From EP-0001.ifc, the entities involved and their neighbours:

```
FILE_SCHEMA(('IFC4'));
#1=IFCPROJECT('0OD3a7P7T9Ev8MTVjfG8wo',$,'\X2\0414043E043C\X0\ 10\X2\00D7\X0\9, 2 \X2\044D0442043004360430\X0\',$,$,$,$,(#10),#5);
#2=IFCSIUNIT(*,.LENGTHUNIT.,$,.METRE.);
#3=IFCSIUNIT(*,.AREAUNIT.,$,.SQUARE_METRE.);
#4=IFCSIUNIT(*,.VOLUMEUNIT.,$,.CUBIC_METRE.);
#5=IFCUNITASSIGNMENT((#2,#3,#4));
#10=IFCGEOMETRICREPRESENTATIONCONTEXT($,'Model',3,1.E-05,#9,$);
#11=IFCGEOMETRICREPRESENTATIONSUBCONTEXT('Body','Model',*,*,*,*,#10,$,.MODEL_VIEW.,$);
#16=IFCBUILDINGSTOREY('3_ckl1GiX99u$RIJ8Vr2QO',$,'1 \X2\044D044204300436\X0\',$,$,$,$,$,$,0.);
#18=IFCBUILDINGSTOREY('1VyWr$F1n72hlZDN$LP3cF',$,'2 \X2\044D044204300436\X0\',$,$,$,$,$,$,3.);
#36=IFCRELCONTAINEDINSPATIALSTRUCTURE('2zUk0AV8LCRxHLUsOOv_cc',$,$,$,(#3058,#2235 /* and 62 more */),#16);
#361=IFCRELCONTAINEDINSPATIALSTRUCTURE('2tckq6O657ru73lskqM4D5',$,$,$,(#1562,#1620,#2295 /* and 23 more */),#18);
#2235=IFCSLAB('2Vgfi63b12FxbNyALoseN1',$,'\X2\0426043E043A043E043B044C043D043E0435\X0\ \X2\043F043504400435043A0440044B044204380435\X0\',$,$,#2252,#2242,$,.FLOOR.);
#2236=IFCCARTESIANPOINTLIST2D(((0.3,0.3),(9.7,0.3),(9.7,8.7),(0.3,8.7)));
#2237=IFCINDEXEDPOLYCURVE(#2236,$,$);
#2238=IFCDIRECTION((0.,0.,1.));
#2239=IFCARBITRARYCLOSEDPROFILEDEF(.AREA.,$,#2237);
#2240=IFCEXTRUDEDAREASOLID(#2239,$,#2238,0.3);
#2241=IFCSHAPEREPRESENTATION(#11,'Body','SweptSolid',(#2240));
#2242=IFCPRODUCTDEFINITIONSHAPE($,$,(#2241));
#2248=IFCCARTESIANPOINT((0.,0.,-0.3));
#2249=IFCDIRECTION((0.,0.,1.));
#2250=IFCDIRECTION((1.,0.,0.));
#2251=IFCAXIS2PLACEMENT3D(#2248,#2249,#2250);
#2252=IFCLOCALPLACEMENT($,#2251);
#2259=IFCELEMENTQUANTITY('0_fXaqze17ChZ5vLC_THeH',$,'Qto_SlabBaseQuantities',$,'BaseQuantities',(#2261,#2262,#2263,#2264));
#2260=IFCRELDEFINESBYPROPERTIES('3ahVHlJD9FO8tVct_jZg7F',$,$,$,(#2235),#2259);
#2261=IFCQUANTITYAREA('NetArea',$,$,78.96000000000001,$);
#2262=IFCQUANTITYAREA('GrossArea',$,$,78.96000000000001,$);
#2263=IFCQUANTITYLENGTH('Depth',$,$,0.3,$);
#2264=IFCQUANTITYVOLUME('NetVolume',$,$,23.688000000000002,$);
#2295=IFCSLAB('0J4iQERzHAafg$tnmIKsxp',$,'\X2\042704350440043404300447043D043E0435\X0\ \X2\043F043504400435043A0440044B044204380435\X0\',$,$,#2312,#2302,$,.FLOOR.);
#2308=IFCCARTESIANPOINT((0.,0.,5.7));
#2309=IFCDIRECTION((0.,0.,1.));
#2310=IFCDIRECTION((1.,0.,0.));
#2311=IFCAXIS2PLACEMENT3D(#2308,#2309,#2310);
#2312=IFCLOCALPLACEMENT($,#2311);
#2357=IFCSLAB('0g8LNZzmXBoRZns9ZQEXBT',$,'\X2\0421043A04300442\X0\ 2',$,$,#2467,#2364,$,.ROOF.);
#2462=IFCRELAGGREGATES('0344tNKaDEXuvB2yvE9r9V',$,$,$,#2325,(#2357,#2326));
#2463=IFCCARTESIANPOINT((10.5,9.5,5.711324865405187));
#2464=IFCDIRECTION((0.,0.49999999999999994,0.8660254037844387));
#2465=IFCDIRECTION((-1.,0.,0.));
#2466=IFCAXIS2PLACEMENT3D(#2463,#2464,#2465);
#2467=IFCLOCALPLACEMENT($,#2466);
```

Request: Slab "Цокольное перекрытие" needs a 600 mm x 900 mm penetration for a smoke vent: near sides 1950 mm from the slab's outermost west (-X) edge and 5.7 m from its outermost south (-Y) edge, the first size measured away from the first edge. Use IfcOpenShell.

```python
import numpy as np
import ifcopenshell
import ifcopenshell.api.feature
import ifcopenshell.api.geometry
import ifcopenshell.api.pset
import ifcopenshell.api.root
import ifcopenshell.geom
import ifcopenshell.util.element
import ifcopenshell.util.placement
import ifcopenshell.util.representation
import ifcopenshell.util.shape
import ifcopenshell.util.unit

model = ifcopenshell.open("EP-0001.ifc")
unit_scale = ifcopenshell.util.unit.calculate_unit_scale(model)
area_scale = ifcopenshell.util.unit.calculate_unit_scale(model, "AREAUNIT")
volume_scale = ifcopenshell.util.unit.calculate_unit_scale(model, "VOLUMEUNIT")
settings = ifcopenshell.geom.settings()


def volume(element):
    """Net volume in cubic metres, openings subtracted."""
    shape = ifcopenshell.geom.create_shape(settings, element)
    return ifcopenshell.util.shape.get_volume(shape.geometry)


slab = model.by_id(2235)
before = volume(slab)

# Extent in the slab's own axes, in metres. The edges named are its -X and -Y sides.
slab_shape = ifcopenshell.geom.create_shape(settings, slab)
vertices = ifcopenshell.util.shape.get_vertices(slab_shape.geometry)
x_min, y_min, bottom = vertices.min(axis=0)
top = vertices[:, 2].max()

opening = ifcopenshell.api.root.create_entity(model, ifc_class="IfcOpeningElement", name="Smoke vent opening", predefined_type="OPENING")
context = ifcopenshell.util.representation.get_context(model, "Model", "Body", "MODEL_VIEW")
width, depth = 0.6, 0.9
outline = [(0.0, 0.0), (width, 0.0), (width, depth), (0.0, depth), (0.0, 0.0)]
# Overshoot both faces by 50 mm so the cut is clean.
shape = ifcopenshell.api.geometry.add_slab_representation(
    model, context=context, depth=top - bottom + 0.1, polyline=outline
)
ifcopenshell.api.geometry.assign_representation(model, product=opening, representation=shape)

matrix = ifcopenshell.util.placement.get_local_placement(slab.ObjectPlacement)
matrix[:, 3] = matrix @ np.append(np.array([x_min + 1.95, y_min + 5.7, bottom - 0.05]) / unit_scale, 1.0)
ifcopenshell.api.geometry.edit_object_placement(model, product=opening, matrix=matrix, is_si=False)
ifcopenshell.api.feature.add_feature(model, feature=opening, element=slab)

after = volume(slab)

# Update the slab's stored quantities.
qto = model.by_id(ifcopenshell.util.element.get_pset(slab, "Qto_SlabBaseQuantities", should_inherit=False)["id"])
ifcopenshell.api.pset.edit_qto(model, qto=qto, properties={
    "NetArea": after / (top - bottom) / area_scale,
    "NetVolume": after / volume_scale,
})

print(f"slab volume {before:.3f} -> {after:.3f} m3")

model.write("EP-0001_rev.ifc")
```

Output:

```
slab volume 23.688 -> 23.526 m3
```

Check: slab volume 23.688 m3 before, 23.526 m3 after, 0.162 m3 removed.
